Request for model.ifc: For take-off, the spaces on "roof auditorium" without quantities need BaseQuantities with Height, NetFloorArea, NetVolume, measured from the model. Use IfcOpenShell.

First a look at what the model holds.

```python
import ifcopenshell
import ifcopenshell.util.element
import ifcopenshell.util.unit

model = ifcopenshell.open("model.ifc")
print(model.schema)
for unit_type in ("LENGTHUNIT", "AREAUNIT", "VOLUMEUNIT"):
    print(unit_type, ifcopenshell.util.unit.calculate_unit_scale(model, unit_type))
storey = next(s for s in model.by_type("IfcBuildingStorey") if s.Name == "roof auditorium")
spaces = [e for e in ifcopenshell.util.element.get_decomposition(storey) if e.is_a("IfcSpace")]
for e in sorted(spaces, key=lambda e: e.id()):
    print(e.id(), e.is_a(), e.Name, list(ifcopenshell.util.element.get_psets(e, qtos_only=True)), sep=" | ")
```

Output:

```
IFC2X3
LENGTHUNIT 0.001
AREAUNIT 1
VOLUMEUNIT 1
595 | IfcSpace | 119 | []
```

```python
import ifcopenshell
import ifcopenshell.api.pset
import ifcopenshell.geom
import ifcopenshell.util.element
import ifcopenshell.util.shape
import ifcopenshell.util.unit

model = ifcopenshell.open("model.ifc")
unit_scale = ifcopenshell.util.unit.calculate_unit_scale(model)
area_scale = ifcopenshell.util.unit.calculate_unit_scale(model, "AREAUNIT")
volume_scale = ifcopenshell.util.unit.calculate_unit_scale(model, "VOLUMEUNIT")
settings = ifcopenshell.geom.settings()

storey = next(s for s in model.by_type("IfcBuildingStorey") if s.Name == "roof auditorium")
spaces = [e for e in ifcopenshell.util.element.get_decomposition(storey) if e.is_a("IfcSpace")]

for e in sorted(spaces, key=lambda e: e.id()):
    if ifcopenshell.util.element.get_psets(e, qtos_only=True, should_inherit=False):
        continue
    # Geometry comes back in metres, in the element's own axes.
    shape = ifcopenshell.geom.create_shape(settings, e)
    values = {
        "Height": ifcopenshell.util.shape.get_z(shape.geometry) / unit_scale,
        "NetFloorArea": ifcopenshell.util.shape.get_footprint_area(shape.geometry) / area_scale,
        "NetVolume": ifcopenshell.util.shape.get_volume(shape.geometry) / volume_scale,
    }
    qto = ifcopenshell.api.pset.add_qto(model, product=e, name="BaseQuantities")
    ifcopenshell.api.pset.edit_qto(model, qto=qto, properties=values)
    print(e.id(), {k: round(v, 3) for k, v in values.items()})

model.write("model_rev.ifc")
```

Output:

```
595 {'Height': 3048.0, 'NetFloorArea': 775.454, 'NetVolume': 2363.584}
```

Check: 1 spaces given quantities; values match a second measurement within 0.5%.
